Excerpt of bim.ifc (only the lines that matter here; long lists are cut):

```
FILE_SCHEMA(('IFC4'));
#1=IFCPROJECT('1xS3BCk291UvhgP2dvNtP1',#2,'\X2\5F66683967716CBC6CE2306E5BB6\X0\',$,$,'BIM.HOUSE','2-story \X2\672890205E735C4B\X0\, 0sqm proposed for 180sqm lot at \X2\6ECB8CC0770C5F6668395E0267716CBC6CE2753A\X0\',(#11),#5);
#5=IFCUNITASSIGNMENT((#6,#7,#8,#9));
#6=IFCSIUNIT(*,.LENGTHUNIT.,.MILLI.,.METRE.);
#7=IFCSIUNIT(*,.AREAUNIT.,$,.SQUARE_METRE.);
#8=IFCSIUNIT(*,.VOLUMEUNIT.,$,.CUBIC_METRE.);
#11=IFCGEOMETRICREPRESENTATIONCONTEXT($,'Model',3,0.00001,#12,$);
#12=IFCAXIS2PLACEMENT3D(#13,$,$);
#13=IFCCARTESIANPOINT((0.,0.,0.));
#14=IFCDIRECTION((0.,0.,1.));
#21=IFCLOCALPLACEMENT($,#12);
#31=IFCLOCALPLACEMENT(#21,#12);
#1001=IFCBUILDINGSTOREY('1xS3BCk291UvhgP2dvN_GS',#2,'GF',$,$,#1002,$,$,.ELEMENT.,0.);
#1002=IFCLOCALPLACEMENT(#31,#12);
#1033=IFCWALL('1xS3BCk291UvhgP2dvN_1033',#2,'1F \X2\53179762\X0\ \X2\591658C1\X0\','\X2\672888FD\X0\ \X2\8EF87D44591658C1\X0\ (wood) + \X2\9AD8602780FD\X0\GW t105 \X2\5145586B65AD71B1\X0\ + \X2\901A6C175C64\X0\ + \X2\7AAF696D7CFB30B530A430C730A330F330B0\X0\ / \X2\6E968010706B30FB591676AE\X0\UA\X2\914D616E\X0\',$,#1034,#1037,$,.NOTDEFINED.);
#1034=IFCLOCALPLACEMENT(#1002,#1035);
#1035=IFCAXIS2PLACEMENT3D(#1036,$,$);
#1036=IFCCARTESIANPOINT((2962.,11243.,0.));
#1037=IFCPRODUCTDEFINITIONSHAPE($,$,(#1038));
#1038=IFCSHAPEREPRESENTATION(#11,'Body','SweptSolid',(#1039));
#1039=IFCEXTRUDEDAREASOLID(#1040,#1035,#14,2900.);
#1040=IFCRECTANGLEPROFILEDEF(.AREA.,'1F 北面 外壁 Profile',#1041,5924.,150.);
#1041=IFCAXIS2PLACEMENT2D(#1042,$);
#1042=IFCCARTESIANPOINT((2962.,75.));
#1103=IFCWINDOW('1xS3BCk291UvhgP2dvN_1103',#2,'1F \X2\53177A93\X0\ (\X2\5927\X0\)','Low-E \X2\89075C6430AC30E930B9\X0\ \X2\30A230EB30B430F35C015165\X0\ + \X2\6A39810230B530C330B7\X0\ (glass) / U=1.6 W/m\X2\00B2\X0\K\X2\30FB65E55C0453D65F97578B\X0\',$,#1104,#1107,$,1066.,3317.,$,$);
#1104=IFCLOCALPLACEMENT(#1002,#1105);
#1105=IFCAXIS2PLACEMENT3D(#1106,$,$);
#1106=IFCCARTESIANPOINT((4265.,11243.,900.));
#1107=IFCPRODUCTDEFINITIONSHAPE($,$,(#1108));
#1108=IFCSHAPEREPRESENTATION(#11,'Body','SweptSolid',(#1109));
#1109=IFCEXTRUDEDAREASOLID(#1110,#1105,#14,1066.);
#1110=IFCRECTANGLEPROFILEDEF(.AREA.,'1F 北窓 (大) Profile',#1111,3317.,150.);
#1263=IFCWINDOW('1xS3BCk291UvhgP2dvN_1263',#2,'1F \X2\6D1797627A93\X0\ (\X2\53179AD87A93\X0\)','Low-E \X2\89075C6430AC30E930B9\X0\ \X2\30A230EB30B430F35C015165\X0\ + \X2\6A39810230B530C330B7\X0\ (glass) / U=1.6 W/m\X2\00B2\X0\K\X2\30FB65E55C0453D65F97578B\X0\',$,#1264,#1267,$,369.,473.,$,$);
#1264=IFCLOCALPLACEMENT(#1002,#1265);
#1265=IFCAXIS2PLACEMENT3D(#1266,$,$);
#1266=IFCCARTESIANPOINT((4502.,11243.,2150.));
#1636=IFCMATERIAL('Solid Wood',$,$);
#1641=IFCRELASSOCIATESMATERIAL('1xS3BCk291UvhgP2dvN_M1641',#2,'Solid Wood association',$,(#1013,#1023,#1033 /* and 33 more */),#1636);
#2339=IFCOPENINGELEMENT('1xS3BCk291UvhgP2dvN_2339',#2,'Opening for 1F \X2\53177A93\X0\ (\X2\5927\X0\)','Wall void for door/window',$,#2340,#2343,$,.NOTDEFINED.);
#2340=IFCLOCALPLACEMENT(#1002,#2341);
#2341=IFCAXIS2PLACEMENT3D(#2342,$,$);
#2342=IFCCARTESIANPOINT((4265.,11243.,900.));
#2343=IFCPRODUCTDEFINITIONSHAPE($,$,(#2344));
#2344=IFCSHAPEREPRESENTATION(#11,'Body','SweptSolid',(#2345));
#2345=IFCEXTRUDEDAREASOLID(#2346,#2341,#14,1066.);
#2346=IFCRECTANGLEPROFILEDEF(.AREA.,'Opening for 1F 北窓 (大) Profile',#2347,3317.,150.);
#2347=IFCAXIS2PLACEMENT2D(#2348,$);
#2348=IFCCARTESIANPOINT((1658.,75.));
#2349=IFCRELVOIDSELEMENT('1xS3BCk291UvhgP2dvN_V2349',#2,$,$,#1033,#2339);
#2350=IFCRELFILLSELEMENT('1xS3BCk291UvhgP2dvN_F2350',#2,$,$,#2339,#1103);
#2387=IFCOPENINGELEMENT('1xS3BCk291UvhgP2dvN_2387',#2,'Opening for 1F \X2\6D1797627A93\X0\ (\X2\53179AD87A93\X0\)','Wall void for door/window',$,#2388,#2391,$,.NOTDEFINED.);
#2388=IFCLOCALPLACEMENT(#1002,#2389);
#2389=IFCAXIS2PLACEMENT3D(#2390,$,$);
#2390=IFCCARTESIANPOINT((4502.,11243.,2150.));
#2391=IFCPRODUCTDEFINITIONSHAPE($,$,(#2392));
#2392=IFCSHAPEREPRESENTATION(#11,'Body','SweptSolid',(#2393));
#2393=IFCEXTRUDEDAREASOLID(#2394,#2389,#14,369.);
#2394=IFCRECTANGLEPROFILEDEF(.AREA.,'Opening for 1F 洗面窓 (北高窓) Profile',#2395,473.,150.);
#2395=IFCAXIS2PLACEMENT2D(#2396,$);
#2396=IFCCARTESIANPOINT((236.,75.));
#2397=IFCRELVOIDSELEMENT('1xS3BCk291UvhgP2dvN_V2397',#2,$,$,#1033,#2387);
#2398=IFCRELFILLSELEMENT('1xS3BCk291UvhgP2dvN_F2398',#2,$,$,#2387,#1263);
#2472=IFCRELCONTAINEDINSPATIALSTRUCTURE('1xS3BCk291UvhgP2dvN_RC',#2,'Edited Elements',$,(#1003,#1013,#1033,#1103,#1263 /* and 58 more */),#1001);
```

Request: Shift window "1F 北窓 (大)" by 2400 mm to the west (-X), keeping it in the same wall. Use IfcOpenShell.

```python
import ifcopenshell
import ifcopenshell.api.geometry
import ifcopenshell.util.placement

model = ifcopenshell.open("bim.ifc")

window = model.by_guid("1xS3BCk291UvhgP2dvN_1103")
opening = window.FillsVoids[0].RelatingOpeningElement
wall = opening.VoidsElements[0].RelatingBuildingElement

wall_matrix = ifcopenshell.util.placement.get_local_placement(wall.ObjectPlacement)
shift = wall_matrix[:3, 0] * -2400.0
before = ifcopenshell.util.placement.get_local_placement(window.ObjectPlacement)[:3, 3].copy()

# The window is not placed relative to its opening, so move both.
for product in (opening, window):
    matrix = ifcopenshell.util.placement.get_local_placement(product.ObjectPlacement)
    matrix[:3, 3] += shift
    ifcopenshell.api.geometry.edit_object_placement(model, product=product, matrix=matrix, is_si=False)

after = ifcopenshell.util.placement.get_local_placement(window.ObjectPlacement)[:3, 3]
print("window moved by", (after - before).round(3) + 0.0)

model.write("bim_updated.ifc")
```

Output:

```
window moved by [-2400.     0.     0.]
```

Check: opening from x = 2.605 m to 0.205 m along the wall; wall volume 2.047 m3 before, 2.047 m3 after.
